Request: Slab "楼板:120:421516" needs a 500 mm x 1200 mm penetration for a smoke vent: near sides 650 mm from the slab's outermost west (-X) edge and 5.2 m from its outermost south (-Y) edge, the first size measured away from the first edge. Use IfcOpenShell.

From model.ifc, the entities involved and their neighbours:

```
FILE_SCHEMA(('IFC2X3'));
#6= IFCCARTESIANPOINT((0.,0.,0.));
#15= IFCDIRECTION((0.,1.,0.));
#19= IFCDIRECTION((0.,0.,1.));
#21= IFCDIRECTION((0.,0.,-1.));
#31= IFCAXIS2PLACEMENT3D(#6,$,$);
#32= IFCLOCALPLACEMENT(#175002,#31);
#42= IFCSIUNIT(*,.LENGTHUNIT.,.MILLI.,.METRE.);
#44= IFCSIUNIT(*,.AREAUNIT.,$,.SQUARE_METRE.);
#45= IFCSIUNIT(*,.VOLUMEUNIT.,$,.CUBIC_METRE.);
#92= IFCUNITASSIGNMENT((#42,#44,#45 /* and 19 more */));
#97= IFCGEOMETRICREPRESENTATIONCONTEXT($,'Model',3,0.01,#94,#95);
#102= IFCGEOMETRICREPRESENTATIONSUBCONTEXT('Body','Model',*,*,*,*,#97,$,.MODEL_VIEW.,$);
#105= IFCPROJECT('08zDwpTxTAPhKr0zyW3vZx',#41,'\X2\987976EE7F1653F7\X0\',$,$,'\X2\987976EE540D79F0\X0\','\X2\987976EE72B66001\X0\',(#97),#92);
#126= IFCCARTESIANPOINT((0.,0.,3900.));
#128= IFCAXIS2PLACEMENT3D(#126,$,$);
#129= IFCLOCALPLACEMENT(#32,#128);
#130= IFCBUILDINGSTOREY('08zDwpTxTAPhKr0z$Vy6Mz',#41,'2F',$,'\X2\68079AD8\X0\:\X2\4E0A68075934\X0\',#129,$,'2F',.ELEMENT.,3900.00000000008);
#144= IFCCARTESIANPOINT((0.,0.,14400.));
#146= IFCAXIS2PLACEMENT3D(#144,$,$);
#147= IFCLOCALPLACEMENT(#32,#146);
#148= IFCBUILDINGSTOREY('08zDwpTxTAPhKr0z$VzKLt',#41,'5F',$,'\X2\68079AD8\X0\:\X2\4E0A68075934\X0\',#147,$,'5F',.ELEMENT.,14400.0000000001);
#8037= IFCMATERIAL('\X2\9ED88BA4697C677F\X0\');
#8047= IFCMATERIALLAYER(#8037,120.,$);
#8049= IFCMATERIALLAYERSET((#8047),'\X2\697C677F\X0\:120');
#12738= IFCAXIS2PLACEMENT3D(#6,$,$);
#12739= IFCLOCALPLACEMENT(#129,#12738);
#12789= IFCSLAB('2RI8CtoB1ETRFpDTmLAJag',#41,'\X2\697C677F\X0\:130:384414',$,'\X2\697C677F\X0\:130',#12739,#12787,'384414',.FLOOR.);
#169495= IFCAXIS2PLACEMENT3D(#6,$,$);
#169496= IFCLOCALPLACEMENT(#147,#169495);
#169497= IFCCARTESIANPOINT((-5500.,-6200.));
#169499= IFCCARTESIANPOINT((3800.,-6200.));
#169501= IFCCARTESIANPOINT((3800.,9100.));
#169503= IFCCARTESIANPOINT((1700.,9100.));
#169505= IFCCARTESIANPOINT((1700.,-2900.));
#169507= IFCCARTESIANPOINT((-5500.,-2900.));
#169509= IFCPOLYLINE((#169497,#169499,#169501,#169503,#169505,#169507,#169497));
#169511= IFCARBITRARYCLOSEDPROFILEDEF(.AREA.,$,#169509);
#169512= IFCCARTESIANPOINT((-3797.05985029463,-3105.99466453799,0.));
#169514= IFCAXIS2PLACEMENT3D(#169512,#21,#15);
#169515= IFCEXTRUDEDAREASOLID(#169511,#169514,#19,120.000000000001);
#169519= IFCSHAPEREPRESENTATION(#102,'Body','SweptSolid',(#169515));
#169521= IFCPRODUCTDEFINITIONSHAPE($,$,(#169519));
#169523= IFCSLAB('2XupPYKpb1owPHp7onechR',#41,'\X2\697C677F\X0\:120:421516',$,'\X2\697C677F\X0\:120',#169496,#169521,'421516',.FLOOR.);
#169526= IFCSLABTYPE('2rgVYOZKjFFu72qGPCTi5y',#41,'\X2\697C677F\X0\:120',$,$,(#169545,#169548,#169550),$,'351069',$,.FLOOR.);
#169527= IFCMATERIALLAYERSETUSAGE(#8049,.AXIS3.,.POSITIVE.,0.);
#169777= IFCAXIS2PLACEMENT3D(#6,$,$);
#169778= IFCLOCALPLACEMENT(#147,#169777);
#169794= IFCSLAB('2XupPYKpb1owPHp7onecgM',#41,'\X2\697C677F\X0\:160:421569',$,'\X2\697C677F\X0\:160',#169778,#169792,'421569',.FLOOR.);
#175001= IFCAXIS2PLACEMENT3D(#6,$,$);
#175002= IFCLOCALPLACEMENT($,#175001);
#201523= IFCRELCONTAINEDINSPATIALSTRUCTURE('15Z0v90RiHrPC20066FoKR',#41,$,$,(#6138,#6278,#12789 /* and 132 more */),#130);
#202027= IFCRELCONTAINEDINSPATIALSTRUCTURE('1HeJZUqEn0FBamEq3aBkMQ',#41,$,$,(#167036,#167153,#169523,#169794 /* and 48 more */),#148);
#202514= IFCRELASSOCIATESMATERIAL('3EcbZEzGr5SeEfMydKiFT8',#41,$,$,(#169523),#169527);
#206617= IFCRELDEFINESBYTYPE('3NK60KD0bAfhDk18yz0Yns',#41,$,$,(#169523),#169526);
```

```python
import numpy as np
import ifcopenshell
import ifcopenshell.api.feature
import ifcopenshell.api.geometry
import ifcopenshell.api.root
import ifcopenshell.geom
import ifcopenshell.util.placement
import ifcopenshell.util.representation
import ifcopenshell.util.shape
import ifcopenshell.util.unit

model = ifcopenshell.open("model.ifc")
unit_scale = ifcopenshell.util.unit.calculate_unit_scale(model)
settings = ifcopenshell.geom.settings()


def volume(element):
    """Net volume in cubic metres, openings subtracted."""
    shape = ifcopenshell.geom.create_shape(settings, element)
    return ifcopenshell.util.shape.get_volume(shape.geometry)


slab = model.by_id(169523)
before = volume(slab)

# Extent in the slab's own axes, in metres. The edges named are its -X and -Y sides.
slab_shape = ifcopenshell.geom.create_shape(settings, slab)
vertices = ifcopenshell.util.shape.get_vertices(slab_shape.geometry)
x_min, y_min, bottom = vertices.min(axis=0)
top = vertices[:, 2].max()

opening = ifcopenshell.api.root.create_entity(model, ifc_class="IfcOpeningElement", name="Smoke vent opening")
context = ifcopenshell.util.representation.get_context(model, "Model", "Body", "MODEL_VIEW")
width, depth = 0.5, 1.2
outline = [(0.0, 0.0), (width, 0.0), (width, depth), (0.0, depth), (0.0, 0.0)]
# Overshoot both faces by 50 mm so the cut is clean.
shape = ifcopenshell.api.geometry.add_slab_representation(
    model, context=context, depth=top - bottom + 0.1, polyline=outline
)
ifcopenshell.api.geometry.assign_representation(model, product=opening, representation=shape)

matrix = ifcopenshell.util.placement.get_local_placement(slab.ObjectPlacement)
matrix[:, 3] = matrix @ np.append(np.array([x_min + 0.65, y_min + 5.2, bottom - 0.05]) / unit_scale, 1.0)
ifcopenshell.api.geometry.edit_object_placement(model, product=opening, matrix=matrix, is_si=False)
ifcopenshell.api.feature.add_feature(model, feature=opening, element=slab)

after = volume(slab)

print(f"slab volume {before:.3f} -> {after:.3f} m3")

model.write("model_rev.ifc")
```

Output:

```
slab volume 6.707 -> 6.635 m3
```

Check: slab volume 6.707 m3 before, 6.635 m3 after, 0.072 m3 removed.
